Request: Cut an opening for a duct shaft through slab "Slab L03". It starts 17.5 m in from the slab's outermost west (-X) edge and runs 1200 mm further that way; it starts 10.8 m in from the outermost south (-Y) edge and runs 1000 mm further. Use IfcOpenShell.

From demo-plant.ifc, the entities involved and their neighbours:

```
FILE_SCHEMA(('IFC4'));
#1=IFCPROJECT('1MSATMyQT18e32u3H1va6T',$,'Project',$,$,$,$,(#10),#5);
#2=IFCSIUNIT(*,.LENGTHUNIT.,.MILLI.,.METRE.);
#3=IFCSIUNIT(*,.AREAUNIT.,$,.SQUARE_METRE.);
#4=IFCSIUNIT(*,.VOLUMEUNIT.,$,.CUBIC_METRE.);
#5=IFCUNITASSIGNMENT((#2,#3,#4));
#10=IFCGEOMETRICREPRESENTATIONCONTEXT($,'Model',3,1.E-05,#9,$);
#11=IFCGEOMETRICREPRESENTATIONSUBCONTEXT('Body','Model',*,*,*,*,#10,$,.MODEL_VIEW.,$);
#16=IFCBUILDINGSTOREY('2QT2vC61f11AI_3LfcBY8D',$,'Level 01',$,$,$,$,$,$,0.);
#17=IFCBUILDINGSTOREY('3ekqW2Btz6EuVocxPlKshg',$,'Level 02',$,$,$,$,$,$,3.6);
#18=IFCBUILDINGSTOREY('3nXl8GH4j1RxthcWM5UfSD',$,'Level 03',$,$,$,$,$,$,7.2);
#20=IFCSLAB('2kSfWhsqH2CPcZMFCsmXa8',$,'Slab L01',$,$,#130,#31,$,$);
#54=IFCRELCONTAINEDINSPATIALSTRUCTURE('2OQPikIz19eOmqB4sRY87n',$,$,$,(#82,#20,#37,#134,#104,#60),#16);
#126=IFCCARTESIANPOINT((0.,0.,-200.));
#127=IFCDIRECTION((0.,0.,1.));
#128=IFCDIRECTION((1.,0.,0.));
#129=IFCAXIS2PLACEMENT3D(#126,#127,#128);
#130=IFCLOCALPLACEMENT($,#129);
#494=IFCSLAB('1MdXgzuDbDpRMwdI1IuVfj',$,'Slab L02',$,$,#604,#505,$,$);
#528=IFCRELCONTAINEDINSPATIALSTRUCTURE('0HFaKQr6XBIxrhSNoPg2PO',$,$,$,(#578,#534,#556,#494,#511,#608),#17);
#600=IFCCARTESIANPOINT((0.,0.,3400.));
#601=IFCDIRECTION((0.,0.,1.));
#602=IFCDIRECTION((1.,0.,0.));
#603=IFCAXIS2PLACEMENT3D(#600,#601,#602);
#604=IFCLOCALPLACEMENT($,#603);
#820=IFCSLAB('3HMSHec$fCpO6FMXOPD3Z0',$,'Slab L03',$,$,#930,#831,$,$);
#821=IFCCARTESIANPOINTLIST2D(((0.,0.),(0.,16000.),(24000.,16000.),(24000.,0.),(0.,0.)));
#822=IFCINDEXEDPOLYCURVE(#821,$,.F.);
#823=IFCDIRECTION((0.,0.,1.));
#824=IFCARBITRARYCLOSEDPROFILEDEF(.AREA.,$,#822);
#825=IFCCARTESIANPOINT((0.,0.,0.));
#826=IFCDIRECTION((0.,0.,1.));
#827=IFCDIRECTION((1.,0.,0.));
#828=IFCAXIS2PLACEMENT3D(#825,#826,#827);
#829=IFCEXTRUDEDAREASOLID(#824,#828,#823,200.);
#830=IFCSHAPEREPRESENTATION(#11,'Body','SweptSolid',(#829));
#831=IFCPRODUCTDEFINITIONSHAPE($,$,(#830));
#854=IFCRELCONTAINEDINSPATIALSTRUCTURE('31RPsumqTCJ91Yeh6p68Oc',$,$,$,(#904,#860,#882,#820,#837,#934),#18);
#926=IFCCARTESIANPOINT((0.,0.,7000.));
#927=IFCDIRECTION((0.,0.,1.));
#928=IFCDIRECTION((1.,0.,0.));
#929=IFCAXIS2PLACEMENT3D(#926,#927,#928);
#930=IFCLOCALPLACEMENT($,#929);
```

```python
import numpy as np
import ifcopenshell
import ifcopenshell.api.feature
import ifcopenshell.api.geometry
import ifcopenshell.api.root
import ifcopenshell.geom
import ifcopenshell.util.placement
import ifcopenshell.util.representation
import ifcopenshell.util.shape
import ifcopenshell.util.unit

model = ifcopenshell.open("demo-plant.ifc")
unit_scale = ifcopenshell.util.unit.calculate_unit_scale(model)
settings = ifcopenshell.geom.settings()


def volume(element):
    """Net volume in cubic metres, openings subtracted."""
    shape = ifcopenshell.geom.create_shape(settings, element)
    return ifcopenshell.util.shape.get_volume(shape.geometry)


slab = model.by_guid("3HMSHec$fCpO6FMXOPD3Z0")
before = volume(slab)

# Extent in the slab's own axes, in metres. The edges named are its -X and -Y sides.
slab_shape = ifcopenshell.geom.create_shape(settings, slab)
vertices = ifcopenshell.util.shape.get_vertices(slab_shape.geometry)
x_min, y_min, bottom = vertices.min(axis=0)
top = vertices[:, 2].max()

opening = ifcopenshell.api.root.create_entity(model, ifc_class="IfcOpeningElement", name="Duct shaft opening", predefined_type="OPENING")
context = ifcopenshell.util.representation.get_context(model, "Model", "Body", "MODEL_VIEW")
width, depth = 1.2, 1
outline = [(0.0, 0.0), (width, 0.0), (width, depth), (0.0, depth), (0.0, 0.0)]
# Overshoot both faces by 50 mm so the cut is clean.
shape = ifcopenshell.api.geometry.add_slab_representation(
    model, context=context, depth=top - bottom + 0.1, polyline=outline
)
ifcopenshell.api.geometry.assign_representation(model, product=opening, representation=shape)

matrix = ifcopenshell.util.placement.get_local_placement(slab.ObjectPlacement)
matrix[:, 3] = matrix @ np.append(np.array([x_min + 17.5, y_min + 10.8, bottom - 0.05]) / unit_scale, 1.0)
ifcopenshell.api.geometry.edit_object_placement(model, product=opening, matrix=matrix, is_si=False)
ifcopenshell.api.feature.add_feature(model, feature=opening, element=slab)

after = volume(slab)

print(f"slab volume {before:.3f} -> {after:.3f} m3")

model.write("demo-plant_rev.ifc")
```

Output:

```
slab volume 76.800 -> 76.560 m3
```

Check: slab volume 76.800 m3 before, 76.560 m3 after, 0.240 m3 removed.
